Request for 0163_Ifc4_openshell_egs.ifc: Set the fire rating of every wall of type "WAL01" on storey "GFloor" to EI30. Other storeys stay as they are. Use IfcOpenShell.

First a look at what the model holds.

```python
import ifcopenshell
import ifcopenshell.util.element

model = ifcopenshell.open("0163_Ifc4_openshell_egs.ifc")
print(model.schema)
storey = next(s for s in model.by_type("IfcBuildingStorey") if s.Name == "GFloor")
walls = [e for e in ifcopenshell.util.element.get_decomposition(storey) if e.is_a("IfcWall")]
seen = {}
for e in walls:
    element_type = ifcopenshell.util.element.get_type(e)
    key = (element_type.Name if element_type != e and element_type else None, ifcopenshell.util.element.get_pset(e, "Pset_WallCommon", "FireRating"))
    seen[key] = seen.get(key, 0) + 1
for (name, value), count in sorted(seen.items(), key=str):
    print(count, "x", name, "|", value)
```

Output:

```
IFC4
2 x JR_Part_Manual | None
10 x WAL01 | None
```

```python
import ifcopenshell
import ifcopenshell.api.pset
import ifcopenshell.util.element

model = ifcopenshell.open("0163_Ifc4_openshell_egs.ifc")

storey = next(s for s in model.by_type("IfcBuildingStorey") if s.Name == "GFloor")
walls = [e for e in ifcopenshell.util.element.get_decomposition(storey) if e.is_a("IfcWall")]

count = 0
for e in walls:
    element_type = ifcopenshell.util.element.get_type(e)
    if element_type in (None, e) or element_type.Name != "WAL01":
        continue
    # add_pset returns the element's existing set when there is one.
    pset = ifcopenshell.api.pset.add_pset(model, product=e, name="Pset_WallCommon")
    ifcopenshell.api.pset.edit_pset(model, pset=pset, properties={"FireRating": "EI30"})
    count += 1

print(count, "walls updated")

model.write("0163_Ifc4_openshell_egs_edited.ifc")
```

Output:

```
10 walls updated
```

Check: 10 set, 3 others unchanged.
